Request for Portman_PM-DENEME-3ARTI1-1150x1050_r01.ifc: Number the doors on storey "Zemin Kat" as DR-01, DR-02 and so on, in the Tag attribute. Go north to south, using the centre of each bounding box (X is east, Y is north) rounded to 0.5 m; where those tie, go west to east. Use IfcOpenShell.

First a look at what the model holds.

```python
import ifcopenshell
import ifcopenshell.util.element
import ifcopenshell.util.placement

model = ifcopenshell.open("Portman_PM-DENEME-3ARTI1-1150x1050_r01.ifc")
print(model.schema)
storey = next(s for s in model.by_type("IfcBuildingStorey") if s.Name == "Zemin Kat")
doors = [e for e in ifcopenshell.util.element.get_decomposition(storey) if e.is_a("IfcDoor")]
for e in sorted(doors, key=lambda e: e.id()):
    origin = ifcopenshell.util.placement.get_local_placement(e.ObjectPlacement)[:3, 3]
    print(e.id(), e.Tag, e.Name, origin.round(2) + 0.0, sep=" | ")
```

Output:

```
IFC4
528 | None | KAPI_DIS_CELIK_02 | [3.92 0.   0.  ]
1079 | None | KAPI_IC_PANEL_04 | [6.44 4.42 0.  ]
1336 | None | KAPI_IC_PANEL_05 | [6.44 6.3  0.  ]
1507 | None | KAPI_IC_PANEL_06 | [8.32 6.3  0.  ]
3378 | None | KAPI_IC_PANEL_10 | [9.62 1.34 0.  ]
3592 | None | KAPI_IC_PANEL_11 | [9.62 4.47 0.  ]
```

```python
import ifcopenshell
import ifcopenshell.geom
import ifcopenshell.util.element
import ifcopenshell.util.shape

model = ifcopenshell.open("Portman_PM-DENEME-3ARTI1-1150x1050_r01.ifc")
settings = ifcopenshell.geom.settings()
settings.set("use-world-coords", True)


def centre(element):
    shape = ifcopenshell.geom.create_shape(settings, element)
    return ifcopenshell.util.shape.get_bbox_centroid(shape.geometry)


storey = next(s for s in model.by_type("IfcBuildingStorey") if s.Name == "Zemin Kat")
doors = [e for e in ifcopenshell.util.element.get_decomposition(storey) if e.is_a("IfcDoor")]

# Insertion points can sit at a corner or the storey origin, so sort by the geometry (in metres).
centres = {e: centre(e) for e in doors}
doors.sort(key=lambda e: (-round(centres[e][1] / 0.5), centres[e][0]))

for i, e in enumerate(doors, start=1):
    number = f"DR-{i:02d}"
    e.Tag = number
    print(e.id(), number)

model.write("Portman_PM-DENEME-3ARTI1-1150x1050_r01_edited.ifc")
```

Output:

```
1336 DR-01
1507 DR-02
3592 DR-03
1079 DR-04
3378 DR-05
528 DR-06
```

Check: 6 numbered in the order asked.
